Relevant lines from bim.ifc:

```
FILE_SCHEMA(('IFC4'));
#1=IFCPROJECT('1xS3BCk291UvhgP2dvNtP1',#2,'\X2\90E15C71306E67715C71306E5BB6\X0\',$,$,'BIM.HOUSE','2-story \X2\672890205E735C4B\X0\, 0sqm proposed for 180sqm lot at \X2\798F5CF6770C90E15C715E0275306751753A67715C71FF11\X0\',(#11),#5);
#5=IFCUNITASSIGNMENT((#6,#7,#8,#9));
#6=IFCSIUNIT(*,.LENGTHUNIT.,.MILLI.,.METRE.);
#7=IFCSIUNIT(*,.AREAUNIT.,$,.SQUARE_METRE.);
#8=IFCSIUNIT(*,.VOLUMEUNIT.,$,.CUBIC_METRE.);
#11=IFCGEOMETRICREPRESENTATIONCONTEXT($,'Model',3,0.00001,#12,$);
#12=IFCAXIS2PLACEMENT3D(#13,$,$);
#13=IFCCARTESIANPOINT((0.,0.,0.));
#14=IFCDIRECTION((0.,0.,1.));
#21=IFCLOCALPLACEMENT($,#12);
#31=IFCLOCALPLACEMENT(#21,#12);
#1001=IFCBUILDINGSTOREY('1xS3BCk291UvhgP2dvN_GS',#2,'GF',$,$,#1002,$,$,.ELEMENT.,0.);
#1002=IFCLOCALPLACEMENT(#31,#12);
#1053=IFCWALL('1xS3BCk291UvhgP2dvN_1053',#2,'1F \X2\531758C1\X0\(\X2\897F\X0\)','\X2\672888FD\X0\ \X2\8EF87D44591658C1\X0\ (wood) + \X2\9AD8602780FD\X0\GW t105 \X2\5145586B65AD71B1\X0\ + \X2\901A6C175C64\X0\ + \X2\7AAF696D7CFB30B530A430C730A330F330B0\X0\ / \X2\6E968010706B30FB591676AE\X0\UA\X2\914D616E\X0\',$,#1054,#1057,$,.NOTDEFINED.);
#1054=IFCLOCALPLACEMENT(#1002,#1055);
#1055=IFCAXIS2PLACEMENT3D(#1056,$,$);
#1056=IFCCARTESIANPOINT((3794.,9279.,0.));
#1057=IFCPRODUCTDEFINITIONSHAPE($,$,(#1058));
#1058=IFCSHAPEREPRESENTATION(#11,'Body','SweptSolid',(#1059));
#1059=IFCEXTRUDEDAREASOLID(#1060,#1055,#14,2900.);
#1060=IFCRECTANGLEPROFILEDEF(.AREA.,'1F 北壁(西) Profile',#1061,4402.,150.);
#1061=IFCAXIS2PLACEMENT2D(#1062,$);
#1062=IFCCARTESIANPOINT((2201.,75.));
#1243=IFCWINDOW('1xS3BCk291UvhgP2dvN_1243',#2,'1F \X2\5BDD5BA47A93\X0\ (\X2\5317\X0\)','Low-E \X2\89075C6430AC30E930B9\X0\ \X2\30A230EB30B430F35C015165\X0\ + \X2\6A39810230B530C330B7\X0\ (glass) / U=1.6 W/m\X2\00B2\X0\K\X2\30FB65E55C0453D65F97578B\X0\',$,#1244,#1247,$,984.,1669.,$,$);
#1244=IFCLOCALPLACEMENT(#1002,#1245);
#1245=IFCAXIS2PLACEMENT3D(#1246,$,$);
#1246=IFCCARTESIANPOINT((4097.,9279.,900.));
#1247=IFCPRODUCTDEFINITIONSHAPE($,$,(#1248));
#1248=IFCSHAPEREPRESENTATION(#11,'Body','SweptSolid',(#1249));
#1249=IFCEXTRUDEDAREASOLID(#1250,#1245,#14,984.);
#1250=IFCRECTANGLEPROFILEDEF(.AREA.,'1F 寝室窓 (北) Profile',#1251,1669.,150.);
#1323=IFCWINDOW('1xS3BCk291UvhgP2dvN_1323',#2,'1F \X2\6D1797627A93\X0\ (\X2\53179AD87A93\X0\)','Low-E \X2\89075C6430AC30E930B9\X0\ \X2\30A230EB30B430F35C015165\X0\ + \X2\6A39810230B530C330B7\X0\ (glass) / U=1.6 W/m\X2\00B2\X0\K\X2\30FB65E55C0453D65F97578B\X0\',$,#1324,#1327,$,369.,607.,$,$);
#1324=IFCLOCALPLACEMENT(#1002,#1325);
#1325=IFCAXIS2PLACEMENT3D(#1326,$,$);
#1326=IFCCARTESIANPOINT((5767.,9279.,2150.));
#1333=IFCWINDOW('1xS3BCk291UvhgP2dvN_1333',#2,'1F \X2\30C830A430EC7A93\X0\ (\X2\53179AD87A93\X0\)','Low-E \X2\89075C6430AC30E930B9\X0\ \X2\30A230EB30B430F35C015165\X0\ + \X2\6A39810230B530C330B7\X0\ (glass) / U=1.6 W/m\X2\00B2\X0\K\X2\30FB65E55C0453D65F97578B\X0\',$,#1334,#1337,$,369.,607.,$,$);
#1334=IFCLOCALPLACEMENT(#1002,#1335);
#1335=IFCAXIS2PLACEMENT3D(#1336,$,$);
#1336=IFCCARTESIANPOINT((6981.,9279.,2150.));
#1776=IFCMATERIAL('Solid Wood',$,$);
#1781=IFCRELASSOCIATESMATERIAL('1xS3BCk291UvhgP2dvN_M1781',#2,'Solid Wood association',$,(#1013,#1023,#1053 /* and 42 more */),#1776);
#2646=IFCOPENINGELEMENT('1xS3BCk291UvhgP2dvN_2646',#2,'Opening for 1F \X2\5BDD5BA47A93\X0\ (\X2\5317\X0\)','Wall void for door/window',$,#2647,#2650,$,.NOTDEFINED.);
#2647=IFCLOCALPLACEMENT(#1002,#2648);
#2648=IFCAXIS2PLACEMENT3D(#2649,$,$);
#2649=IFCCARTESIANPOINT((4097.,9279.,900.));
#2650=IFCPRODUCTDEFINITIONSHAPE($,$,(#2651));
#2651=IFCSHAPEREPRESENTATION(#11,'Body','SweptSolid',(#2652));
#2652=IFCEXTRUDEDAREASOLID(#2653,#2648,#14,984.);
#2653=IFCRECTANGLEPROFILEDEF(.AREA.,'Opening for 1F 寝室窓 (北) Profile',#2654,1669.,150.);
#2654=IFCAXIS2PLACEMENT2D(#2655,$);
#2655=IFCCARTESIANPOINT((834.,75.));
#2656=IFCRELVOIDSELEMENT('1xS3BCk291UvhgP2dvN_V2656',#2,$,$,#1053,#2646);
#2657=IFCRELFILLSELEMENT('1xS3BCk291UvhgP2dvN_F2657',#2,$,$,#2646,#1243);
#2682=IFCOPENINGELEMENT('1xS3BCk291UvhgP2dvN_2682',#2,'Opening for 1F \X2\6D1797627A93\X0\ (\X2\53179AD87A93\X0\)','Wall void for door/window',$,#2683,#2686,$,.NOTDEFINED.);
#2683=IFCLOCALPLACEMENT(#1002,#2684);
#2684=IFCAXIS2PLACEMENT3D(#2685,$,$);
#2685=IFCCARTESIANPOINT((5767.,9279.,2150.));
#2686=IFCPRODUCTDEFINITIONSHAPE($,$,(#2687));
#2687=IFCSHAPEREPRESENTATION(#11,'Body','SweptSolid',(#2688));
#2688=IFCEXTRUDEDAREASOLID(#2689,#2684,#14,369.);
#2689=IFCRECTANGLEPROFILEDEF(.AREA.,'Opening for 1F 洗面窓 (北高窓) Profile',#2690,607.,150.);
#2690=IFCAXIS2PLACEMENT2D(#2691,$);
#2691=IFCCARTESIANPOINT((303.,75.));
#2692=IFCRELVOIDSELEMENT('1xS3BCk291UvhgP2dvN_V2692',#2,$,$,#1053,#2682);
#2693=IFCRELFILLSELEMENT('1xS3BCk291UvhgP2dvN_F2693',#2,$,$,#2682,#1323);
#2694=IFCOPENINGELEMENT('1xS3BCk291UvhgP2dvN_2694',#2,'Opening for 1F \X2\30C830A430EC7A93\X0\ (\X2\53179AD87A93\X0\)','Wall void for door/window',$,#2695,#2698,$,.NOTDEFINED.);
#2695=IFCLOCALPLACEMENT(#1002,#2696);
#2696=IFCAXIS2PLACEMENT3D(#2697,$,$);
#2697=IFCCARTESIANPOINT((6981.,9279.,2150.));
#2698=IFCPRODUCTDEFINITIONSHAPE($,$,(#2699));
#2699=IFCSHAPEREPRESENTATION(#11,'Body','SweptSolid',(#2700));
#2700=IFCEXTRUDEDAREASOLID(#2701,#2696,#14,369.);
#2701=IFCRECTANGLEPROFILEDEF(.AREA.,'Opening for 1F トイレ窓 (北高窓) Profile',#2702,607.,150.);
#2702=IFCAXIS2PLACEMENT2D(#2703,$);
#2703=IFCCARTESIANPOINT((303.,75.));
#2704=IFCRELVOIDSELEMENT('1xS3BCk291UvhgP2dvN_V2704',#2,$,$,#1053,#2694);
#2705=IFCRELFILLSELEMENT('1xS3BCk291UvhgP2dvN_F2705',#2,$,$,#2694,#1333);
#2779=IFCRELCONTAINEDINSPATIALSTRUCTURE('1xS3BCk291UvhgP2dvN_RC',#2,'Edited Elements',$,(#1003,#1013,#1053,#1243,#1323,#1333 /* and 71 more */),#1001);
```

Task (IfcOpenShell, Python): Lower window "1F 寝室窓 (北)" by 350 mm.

```python
import numpy as np
import ifcopenshell
import ifcopenshell.api.geometry
import ifcopenshell.util.placement
import ifcopenshell.util.unit

model = ifcopenshell.open("bim.ifc")
unit_scale = ifcopenshell.util.unit.calculate_unit_scale(model)

window = model.by_guid("1xS3BCk291UvhgP2dvN_1243")
opening = window.FillsVoids[0].RelatingOpeningElement
dz = -350.0

shift = np.array([0.0, 0.0, dz])
# The window is not placed relative to its opening, so move both.
for product in (opening, window):
    matrix = ifcopenshell.util.placement.get_local_placement(product.ObjectPlacement)
    matrix[:3, 3] += shift
    ifcopenshell.api.geometry.edit_object_placement(model, product=product, matrix=matrix, is_si=False)

print(f"moved by {dz * unit_scale:+.3f} m")

model.write("bim_v2.ifc")
```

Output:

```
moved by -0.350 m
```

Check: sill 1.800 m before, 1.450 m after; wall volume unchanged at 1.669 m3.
